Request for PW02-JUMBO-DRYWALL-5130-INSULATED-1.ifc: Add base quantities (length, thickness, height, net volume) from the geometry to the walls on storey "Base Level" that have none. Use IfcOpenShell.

First a look at what the model holds.

```python
import ifcopenshell
import ifcopenshell.util.element
import ifcopenshell.util.unit

model = ifcopenshell.open("PW02-JUMBO-DRYWALL-5130-INSULATED-1.ifc")
print(model.schema)
for unit_type in ("LENGTHUNIT", "AREAUNIT", "VOLUMEUNIT"):
    print(unit_type, ifcopenshell.util.unit.calculate_unit_scale(model, unit_type))
storey = next(s for s in model.by_type("IfcBuildingStorey") if s.Name == "Base Level")
walls = [e for e in ifcopenshell.util.element.get_decomposition(storey) if e.is_a("IfcWall")]
for e in sorted(walls, key=lambda e: e.id()):
    print(e.id(), e.is_a(), e.Name, list(ifcopenshell.util.element.get_psets(e, qtos_only=True)), sep=" | ")
```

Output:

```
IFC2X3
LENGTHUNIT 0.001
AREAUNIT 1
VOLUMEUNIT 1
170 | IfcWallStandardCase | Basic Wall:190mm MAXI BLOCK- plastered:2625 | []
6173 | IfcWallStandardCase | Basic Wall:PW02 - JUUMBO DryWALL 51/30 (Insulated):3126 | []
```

```python
import ifcopenshell
import ifcopenshell.api.pset
import ifcopenshell.geom
import ifcopenshell.util.element
import ifcopenshell.util.shape
import ifcopenshell.util.unit

model = ifcopenshell.open("PW02-JUMBO-DRYWALL-5130-INSULATED-1.ifc")
unit_scale = ifcopenshell.util.unit.calculate_unit_scale(model)
volume_scale = ifcopenshell.util.unit.calculate_unit_scale(model, "VOLUMEUNIT")
settings = ifcopenshell.geom.settings()

storey = next(s for s in model.by_type("IfcBuildingStorey") if s.Name == "Base Level")
walls = [e for e in ifcopenshell.util.element.get_decomposition(storey) if e.is_a("IfcWall")]

for e in sorted(walls, key=lambda e: e.id()):
    if ifcopenshell.util.element.get_psets(e, qtos_only=True, should_inherit=False):
        continue
    # Geometry comes back in metres, in the element's own axes.
    shape = ifcopenshell.geom.create_shape(settings, e)
    values = {
        "Length": ifcopenshell.util.shape.get_x(shape.geometry) / unit_scale,
        "Width": ifcopenshell.util.shape.get_y(shape.geometry) / unit_scale,
        "Height": ifcopenshell.util.shape.get_z(shape.geometry) / unit_scale,
        "NetVolume": ifcopenshell.util.shape.get_volume(shape.geometry) / volume_scale,
    }
    qto = ifcopenshell.api.pset.add_qto(model, product=e, name="BaseQuantities")
    ifcopenshell.api.pset.edit_qto(model, qto=qto, properties=values)
    print(e.id(), {k: round(v, 3) for k, v in values.items()})

model.write("PW02-JUMBO-DRYWALL-5130-INSULATED-1_updated.ifc")
```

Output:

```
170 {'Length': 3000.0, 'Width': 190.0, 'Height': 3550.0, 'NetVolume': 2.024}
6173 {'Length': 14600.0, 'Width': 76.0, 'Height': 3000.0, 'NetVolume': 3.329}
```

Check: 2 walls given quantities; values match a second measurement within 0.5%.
